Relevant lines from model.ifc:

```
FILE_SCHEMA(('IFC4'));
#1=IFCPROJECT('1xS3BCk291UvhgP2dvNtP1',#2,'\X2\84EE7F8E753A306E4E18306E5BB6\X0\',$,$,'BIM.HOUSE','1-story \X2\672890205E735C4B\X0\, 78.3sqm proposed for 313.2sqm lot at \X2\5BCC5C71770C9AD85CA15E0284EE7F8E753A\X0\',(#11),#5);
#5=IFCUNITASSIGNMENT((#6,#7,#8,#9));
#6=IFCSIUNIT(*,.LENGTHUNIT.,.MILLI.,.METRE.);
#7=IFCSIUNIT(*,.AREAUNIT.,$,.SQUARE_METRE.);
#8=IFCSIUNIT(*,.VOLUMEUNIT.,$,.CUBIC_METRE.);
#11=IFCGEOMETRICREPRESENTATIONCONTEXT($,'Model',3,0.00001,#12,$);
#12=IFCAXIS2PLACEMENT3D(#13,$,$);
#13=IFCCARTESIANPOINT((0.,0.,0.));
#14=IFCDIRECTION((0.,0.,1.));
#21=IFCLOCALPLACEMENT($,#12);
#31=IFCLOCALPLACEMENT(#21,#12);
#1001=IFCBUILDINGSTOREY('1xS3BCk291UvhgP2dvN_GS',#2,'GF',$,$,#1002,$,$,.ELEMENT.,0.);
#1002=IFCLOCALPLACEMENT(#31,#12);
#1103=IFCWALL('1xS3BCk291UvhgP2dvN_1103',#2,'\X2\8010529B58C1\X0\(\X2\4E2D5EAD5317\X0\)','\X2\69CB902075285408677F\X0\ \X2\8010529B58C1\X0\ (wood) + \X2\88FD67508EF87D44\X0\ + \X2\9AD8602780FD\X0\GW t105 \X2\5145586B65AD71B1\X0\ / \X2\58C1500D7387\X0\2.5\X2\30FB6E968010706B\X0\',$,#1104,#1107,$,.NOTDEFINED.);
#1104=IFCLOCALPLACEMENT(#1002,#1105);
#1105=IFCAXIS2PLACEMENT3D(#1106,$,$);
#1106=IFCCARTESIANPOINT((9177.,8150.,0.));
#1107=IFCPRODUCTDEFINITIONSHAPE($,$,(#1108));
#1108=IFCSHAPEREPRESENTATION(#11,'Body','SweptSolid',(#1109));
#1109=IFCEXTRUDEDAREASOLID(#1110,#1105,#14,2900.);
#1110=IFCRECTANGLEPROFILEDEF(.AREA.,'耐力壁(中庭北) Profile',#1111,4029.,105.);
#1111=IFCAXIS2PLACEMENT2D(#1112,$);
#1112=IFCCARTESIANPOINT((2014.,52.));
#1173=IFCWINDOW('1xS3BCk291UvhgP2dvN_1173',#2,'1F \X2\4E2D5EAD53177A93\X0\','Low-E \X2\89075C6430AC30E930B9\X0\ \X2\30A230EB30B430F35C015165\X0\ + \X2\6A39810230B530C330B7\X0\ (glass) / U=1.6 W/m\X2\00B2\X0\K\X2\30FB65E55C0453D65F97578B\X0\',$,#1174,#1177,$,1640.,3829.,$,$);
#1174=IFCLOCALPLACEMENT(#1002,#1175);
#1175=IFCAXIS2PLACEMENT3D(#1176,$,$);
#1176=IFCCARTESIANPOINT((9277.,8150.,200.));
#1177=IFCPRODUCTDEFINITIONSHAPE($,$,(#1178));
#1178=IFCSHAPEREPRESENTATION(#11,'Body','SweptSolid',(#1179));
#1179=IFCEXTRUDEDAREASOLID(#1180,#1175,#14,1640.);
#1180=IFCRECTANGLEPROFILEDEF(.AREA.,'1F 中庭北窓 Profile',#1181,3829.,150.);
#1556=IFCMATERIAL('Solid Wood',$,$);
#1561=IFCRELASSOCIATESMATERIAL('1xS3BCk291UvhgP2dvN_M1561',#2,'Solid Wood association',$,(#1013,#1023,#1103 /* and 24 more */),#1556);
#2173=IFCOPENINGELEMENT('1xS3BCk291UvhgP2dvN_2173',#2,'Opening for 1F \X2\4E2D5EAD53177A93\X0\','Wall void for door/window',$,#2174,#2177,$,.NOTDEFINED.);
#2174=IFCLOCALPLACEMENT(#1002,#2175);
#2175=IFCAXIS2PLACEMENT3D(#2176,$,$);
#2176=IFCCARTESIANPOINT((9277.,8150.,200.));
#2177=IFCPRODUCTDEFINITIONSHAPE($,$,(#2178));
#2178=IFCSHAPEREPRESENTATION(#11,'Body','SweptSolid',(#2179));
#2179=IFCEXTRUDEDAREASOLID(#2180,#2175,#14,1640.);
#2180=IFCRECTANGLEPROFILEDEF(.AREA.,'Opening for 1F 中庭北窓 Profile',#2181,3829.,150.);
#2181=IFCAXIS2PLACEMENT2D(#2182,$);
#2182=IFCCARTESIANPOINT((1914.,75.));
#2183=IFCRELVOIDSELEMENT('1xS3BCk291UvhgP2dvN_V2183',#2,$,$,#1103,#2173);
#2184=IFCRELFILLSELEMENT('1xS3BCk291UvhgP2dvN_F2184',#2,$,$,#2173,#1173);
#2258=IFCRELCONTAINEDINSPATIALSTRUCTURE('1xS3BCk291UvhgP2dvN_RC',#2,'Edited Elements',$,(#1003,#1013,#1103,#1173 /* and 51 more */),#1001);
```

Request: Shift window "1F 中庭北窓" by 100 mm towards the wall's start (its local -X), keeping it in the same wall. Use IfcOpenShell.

```python
import ifcopenshell
import ifcopenshell.api.geometry
import ifcopenshell.util.placement

model = ifcopenshell.open("model.ifc")

window = model.by_guid("1xS3BCk291UvhgP2dvN_1173")
opening = window.FillsVoids[0].RelatingOpeningElement
wall = opening.VoidsElements[0].RelatingBuildingElement

wall_matrix = ifcopenshell.util.placement.get_local_placement(wall.ObjectPlacement)
shift = wall_matrix[:3, 0] * -100.0
before = ifcopenshell.util.placement.get_local_placement(window.ObjectPlacement)[:3, 3].copy()

# The window is not placed relative to its opening, so move both.
for product in (opening, window):
    matrix = ifcopenshell.util.placement.get_local_placement(product.ObjectPlacement)
    matrix[:3, 3] += shift
    ifcopenshell.api.geometry.edit_object_placement(model, product=product, matrix=matrix, is_si=False)

after = ifcopenshell.util.placement.get_local_placement(window.ObjectPlacement)[:3, 3]
print("window moved by", (after - before).round(3) + 0.0)

model.write("model_rev.ifc")
```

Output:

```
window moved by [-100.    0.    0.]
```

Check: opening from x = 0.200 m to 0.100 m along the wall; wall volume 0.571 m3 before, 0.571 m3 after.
